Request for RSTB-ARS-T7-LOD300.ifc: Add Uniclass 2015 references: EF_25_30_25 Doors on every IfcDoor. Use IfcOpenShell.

First a look at what the model holds.

```python
import ifcopenshell

model = ifcopenshell.open("RSTB-ARS-T7-LOD300.ifc")
print(model.schema)
print("classifications:", [c.Name for c in model.by_type("IfcClassification")])
for ifc_class in ("IfcDoor", "IfcRoof", "IfcStair", "IfcWall", "IfcWindow"):
    print(ifc_class, len(model.by_type(ifc_class)))
```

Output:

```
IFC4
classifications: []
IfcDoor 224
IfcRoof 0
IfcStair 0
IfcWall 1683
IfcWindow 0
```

```python
import ifcopenshell
import ifcopenshell.api.classification

model = ifcopenshell.open("RSTB-ARS-T7-LOD300.ifc")

system = ifcopenshell.api.classification.add_classification(model, classification="Uniclass 2015")

codes = {
    "IfcDoor": ("EF_25_30_25", "Doors"),
}
for ifc_class, (code, name) in codes.items():
    products = model.by_type(ifc_class)
    ifcopenshell.api.classification.add_reference(
        model, products=products, classification=system, identification=code, name=name
    )
    print(code, len(products))

model.write("RSTB-ARS-T7-LOD300_edited.ifc")
```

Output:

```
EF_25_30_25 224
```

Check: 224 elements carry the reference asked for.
